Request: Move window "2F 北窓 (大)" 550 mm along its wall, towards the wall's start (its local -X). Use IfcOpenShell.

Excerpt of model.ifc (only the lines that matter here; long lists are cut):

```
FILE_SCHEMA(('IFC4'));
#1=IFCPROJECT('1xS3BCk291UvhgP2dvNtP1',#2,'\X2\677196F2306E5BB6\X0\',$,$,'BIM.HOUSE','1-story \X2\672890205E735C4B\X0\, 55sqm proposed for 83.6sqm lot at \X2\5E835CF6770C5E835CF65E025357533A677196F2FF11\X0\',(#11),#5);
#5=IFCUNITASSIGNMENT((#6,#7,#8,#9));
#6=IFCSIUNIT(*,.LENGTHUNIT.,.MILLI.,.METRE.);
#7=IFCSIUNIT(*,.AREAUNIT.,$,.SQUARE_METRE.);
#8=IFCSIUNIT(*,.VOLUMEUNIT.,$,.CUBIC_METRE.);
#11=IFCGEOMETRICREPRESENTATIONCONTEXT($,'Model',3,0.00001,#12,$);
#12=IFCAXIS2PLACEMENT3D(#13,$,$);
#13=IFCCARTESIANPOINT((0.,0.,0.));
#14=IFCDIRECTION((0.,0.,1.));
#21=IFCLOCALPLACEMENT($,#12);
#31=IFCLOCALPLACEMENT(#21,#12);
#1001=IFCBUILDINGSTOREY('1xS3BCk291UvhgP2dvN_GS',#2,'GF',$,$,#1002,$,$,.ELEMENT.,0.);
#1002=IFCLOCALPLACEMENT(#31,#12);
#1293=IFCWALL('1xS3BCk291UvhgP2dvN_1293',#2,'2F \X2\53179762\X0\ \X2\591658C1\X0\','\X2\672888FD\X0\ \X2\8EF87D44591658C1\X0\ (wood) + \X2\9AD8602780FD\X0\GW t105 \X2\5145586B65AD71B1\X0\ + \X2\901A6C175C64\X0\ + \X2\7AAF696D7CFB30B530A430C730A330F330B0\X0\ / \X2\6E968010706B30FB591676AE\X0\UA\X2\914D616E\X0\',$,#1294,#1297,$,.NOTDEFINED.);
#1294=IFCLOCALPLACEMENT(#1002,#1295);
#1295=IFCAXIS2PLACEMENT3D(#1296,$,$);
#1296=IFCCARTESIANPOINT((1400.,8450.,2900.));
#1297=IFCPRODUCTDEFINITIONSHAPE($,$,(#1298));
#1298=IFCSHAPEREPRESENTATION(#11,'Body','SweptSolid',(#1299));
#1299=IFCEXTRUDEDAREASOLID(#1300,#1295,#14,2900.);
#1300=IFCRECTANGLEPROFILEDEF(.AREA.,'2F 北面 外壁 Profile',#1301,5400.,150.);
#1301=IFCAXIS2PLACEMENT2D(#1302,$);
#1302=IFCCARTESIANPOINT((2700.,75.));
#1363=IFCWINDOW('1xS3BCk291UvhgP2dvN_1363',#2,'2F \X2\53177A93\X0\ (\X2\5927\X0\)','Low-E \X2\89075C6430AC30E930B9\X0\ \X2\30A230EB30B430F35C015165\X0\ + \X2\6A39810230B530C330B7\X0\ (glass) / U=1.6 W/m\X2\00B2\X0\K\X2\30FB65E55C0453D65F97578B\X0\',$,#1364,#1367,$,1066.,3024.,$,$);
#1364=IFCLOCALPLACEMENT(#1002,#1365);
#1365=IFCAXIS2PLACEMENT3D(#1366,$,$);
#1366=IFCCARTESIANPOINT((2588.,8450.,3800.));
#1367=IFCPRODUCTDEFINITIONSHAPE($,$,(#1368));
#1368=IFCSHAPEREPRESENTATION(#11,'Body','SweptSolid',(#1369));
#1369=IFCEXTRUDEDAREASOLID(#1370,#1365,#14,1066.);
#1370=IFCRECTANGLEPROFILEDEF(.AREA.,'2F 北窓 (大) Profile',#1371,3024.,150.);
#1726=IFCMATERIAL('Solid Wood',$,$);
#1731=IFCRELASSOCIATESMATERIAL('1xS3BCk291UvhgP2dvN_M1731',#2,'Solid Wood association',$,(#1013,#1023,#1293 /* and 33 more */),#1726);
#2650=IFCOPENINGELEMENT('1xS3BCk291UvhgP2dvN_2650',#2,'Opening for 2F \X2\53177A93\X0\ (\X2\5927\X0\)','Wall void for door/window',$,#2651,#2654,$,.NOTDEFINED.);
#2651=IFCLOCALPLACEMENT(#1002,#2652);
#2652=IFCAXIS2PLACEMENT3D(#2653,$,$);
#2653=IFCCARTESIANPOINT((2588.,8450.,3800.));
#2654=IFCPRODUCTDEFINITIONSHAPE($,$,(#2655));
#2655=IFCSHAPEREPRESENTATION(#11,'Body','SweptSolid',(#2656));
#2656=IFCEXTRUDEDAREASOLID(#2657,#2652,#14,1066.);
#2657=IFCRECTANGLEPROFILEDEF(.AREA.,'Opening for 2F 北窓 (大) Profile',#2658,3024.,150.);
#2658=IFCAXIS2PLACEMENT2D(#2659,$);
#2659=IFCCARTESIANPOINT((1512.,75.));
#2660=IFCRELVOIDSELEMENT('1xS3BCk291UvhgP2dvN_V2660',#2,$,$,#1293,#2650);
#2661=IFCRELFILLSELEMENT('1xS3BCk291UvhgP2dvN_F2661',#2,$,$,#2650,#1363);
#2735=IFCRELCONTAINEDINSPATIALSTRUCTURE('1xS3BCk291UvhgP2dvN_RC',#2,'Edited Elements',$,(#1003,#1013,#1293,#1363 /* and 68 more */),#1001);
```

```python
import ifcopenshell
import ifcopenshell.api.geometry
import ifcopenshell.util.placement
import ifcopenshell.util.unit

model = ifcopenshell.open("model.ifc")
unit_scale = ifcopenshell.util.unit.calculate_unit_scale(model)

window = model.by_guid("1xS3BCk291UvhgP2dvN_1363")
opening = window.FillsVoids[0].RelatingOpeningElement
wall = opening.VoidsElements[0].RelatingBuildingElement

wall_matrix = ifcopenshell.util.placement.get_local_placement(wall.ObjectPlacement)
shift = wall_matrix[:3, 0] * -0.55 / unit_scale
before = ifcopenshell.util.placement.get_local_placement(window.ObjectPlacement)[:3, 3].copy()

# The window is not placed relative to its opening, so move both.
for product in (opening, window):
    matrix = ifcopenshell.util.placement.get_local_placement(product.ObjectPlacement)
    matrix[:3, 3] += shift
    ifcopenshell.api.geometry.edit_object_placement(model, product=product, matrix=matrix, is_si=False)

after = ifcopenshell.util.placement.get_local_placement(window.ObjectPlacement)[:3, 3]
print("window moved by", (after - before).round(3) + 0.0)

model.write("model_edited.ifc")
```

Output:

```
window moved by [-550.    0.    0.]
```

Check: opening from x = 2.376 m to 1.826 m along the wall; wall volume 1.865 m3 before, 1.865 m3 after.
